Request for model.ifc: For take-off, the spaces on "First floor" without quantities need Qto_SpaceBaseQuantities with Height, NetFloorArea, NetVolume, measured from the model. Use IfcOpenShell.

First a look at what the model holds.

```python
import ifcopenshell
import ifcopenshell.util.element
import ifcopenshell.util.unit

model = ifcopenshell.open("model.ifc")
print(model.schema)
for unit_type in ("LENGTHUNIT", "AREAUNIT", "VOLUMEUNIT"):
    print(unit_type, ifcopenshell.util.unit.calculate_unit_scale(model, unit_type))
storey = next(s for s in model.by_type("IfcBuildingStorey") if s.Name == "First floor")
spaces = [e for e in ifcopenshell.util.element.get_decomposition(storey) if e.is_a("IfcSpace")]
for e in sorted(spaces, key=lambda e: e.id()):
    print(e.id(), e.is_a(), e.Name, list(ifcopenshell.util.element.get_psets(e, qtos_only=True)), sep=" | ")
```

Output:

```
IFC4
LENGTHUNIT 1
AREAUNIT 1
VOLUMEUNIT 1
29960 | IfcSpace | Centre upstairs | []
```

```python
import ifcopenshell
import ifcopenshell.api.pset
import ifcopenshell.geom
import ifcopenshell.util.element
import ifcopenshell.util.shape
import ifcopenshell.util.unit

model = ifcopenshell.open("model.ifc")
unit_scale = ifcopenshell.util.unit.calculate_unit_scale(model)
area_scale = ifcopenshell.util.unit.calculate_unit_scale(model, "AREAUNIT")
volume_scale = ifcopenshell.util.unit.calculate_unit_scale(model, "VOLUMEUNIT")
settings = ifcopenshell.geom.settings()

storey = next(s for s in model.by_type("IfcBuildingStorey") if s.Name == "First floor")
spaces = [e for e in ifcopenshell.util.element.get_decomposition(storey) if e.is_a("IfcSpace")]

for e in sorted(spaces, key=lambda e: e.id()):
    if ifcopenshell.util.element.get_psets(e, qtos_only=True, should_inherit=False):
        continue
    # Geometry comes back in metres, in the element's own axes.
    shape = ifcopenshell.geom.create_shape(settings, e)
    values = {
        "Height": ifcopenshell.util.shape.get_z(shape.geometry) / unit_scale,
        "NetFloorArea": ifcopenshell.util.shape.get_footprint_area(shape.geometry) / area_scale,
        "NetVolume": ifcopenshell.util.shape.get_volume(shape.geometry) / volume_scale,
    }
    qto = ifcopenshell.api.pset.add_qto(model, product=e, name="Qto_SpaceBaseQuantities")
    ifcopenshell.api.pset.edit_qto(model, qto=qto, properties=values)
    print(e.id(), {k: round(v, 3) for k, v in values.items()})

model.write("model_edited.ifc")
```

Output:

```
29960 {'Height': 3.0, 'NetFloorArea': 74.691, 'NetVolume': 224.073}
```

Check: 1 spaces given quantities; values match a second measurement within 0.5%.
